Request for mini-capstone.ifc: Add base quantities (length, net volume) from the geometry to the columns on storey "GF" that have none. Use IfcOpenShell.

First a look at what the model holds.

```python
import ifcopenshell
import ifcopenshell.util.element
import ifcopenshell.util.unit

model = ifcopenshell.open("mini-capstone.ifc")
print(model.schema)
for unit_type in ("LENGTHUNIT", "AREAUNIT", "VOLUMEUNIT"):
    print(unit_type, ifcopenshell.util.unit.calculate_unit_scale(model, unit_type))
storey = next(s for s in model.by_type("IfcBuildingStorey") if s.Name == "GF")
columns = [e for e in ifcopenshell.util.element.get_decomposition(storey) if e.is_a("IfcColumn")]
for e in sorted(columns, key=lambda e: e.id()):
    print(e.id(), e.is_a(), e.Name, list(ifcopenshell.util.element.get_psets(e, qtos_only=True)), sep=" | ")
```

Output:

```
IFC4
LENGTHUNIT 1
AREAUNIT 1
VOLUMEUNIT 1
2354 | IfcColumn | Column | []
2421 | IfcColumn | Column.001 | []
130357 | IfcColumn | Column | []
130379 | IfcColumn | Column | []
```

```python
import ifcopenshell
import ifcopenshell.api.pset
import ifcopenshell.geom
import ifcopenshell.util.element
import ifcopenshell.util.shape
import ifcopenshell.util.unit

model = ifcopenshell.open("mini-capstone.ifc")
unit_scale = ifcopenshell.util.unit.calculate_unit_scale(model)
volume_scale = ifcopenshell.util.unit.calculate_unit_scale(model, "VOLUMEUNIT")
settings = ifcopenshell.geom.settings()

storey = next(s for s in model.by_type("IfcBuildingStorey") if s.Name == "GF")
columns = [e for e in ifcopenshell.util.element.get_decomposition(storey) if e.is_a("IfcColumn")]

for e in sorted(columns, key=lambda e: e.id()):
    if ifcopenshell.util.element.get_psets(e, qtos_only=True, should_inherit=False):
        continue
    # Geometry comes back in metres, in the element's own axes.
    shape = ifcopenshell.geom.create_shape(settings, e)
    values = {
        "Length": ifcopenshell.util.shape.get_z(shape.geometry) / unit_scale,
        "NetVolume": ifcopenshell.util.shape.get_volume(shape.geometry) / volume_scale,
    }
    qto = ifcopenshell.api.pset.add_qto(model, product=e, name="Qto_ColumnBaseQuantities")
    ifcopenshell.api.pset.edit_qto(model, qto=qto, properties=values)
    print(e.id(), {k: round(v, 3) for k, v in values.items()})

model.write("mini-capstone-out.ifc")
```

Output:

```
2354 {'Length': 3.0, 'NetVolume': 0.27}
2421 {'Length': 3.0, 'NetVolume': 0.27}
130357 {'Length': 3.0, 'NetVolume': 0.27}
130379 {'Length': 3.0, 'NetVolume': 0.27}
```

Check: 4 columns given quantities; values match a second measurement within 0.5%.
